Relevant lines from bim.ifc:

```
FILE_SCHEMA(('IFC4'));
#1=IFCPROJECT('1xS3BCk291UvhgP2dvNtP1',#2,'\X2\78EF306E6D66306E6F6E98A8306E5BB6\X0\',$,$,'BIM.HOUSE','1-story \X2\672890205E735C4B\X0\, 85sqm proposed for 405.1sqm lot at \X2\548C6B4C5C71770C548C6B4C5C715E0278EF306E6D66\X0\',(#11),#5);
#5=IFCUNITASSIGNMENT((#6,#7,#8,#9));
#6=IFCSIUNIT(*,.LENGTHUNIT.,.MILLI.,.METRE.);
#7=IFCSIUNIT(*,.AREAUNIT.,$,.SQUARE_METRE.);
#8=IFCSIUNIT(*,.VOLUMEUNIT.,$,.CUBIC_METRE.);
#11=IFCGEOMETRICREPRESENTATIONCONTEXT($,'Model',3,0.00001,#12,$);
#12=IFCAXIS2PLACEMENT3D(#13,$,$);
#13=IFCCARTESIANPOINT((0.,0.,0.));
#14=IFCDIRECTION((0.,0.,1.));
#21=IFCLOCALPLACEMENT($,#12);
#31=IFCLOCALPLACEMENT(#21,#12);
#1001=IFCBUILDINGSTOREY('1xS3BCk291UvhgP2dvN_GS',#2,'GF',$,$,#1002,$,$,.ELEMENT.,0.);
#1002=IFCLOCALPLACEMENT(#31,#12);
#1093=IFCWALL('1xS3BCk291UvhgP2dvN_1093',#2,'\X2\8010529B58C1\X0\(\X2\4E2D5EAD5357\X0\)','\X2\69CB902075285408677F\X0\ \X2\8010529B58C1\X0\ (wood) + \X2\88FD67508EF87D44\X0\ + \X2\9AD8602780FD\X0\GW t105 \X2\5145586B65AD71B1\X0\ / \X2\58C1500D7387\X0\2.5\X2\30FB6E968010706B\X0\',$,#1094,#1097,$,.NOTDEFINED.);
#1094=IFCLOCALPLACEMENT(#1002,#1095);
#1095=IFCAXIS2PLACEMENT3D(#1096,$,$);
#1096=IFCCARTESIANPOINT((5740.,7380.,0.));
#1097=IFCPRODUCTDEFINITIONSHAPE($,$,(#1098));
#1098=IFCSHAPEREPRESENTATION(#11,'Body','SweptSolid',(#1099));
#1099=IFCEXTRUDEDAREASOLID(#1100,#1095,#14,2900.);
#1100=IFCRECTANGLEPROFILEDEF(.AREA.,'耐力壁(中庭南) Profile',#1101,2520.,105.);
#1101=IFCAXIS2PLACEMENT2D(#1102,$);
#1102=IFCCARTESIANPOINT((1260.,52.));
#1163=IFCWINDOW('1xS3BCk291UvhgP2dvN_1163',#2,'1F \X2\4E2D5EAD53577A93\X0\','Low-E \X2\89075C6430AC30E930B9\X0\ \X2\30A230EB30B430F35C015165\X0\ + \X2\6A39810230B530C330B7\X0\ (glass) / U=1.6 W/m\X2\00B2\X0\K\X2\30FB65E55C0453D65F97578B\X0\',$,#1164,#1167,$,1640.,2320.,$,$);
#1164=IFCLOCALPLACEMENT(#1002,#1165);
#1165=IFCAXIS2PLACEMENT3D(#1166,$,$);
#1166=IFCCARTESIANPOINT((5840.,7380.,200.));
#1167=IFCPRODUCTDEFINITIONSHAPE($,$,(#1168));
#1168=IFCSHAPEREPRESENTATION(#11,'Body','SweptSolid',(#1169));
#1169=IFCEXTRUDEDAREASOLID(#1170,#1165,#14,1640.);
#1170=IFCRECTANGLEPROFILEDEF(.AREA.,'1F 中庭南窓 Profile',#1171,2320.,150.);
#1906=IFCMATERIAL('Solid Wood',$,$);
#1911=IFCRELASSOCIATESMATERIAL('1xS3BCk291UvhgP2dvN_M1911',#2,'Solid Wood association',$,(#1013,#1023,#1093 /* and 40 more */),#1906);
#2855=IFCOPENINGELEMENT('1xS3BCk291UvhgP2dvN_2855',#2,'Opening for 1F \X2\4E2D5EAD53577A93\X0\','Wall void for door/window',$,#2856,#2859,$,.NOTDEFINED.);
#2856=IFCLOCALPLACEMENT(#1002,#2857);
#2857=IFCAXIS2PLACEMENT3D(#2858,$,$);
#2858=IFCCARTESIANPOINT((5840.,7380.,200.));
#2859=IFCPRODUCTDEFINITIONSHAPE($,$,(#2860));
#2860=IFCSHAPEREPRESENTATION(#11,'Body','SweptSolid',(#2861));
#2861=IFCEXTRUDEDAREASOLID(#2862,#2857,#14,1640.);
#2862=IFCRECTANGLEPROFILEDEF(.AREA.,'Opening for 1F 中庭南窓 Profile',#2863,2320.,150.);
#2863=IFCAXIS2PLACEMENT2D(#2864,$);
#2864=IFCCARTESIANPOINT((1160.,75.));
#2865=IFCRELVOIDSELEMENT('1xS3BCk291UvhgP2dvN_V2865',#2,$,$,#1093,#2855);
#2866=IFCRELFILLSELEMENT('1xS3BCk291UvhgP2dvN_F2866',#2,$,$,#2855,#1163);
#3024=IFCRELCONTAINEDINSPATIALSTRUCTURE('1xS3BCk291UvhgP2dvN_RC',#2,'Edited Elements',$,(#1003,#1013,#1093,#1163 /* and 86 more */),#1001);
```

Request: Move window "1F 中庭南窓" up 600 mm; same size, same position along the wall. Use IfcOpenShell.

```python
import numpy as np
import ifcopenshell
import ifcopenshell.api.geometry
import ifcopenshell.util.placement
import ifcopenshell.util.unit

model = ifcopenshell.open("bim.ifc")
unit_scale = ifcopenshell.util.unit.calculate_unit_scale(model)

window = model.by_guid("1xS3BCk291UvhgP2dvN_1163")
opening = window.FillsVoids[0].RelatingOpeningElement
dz = 0.6 / unit_scale

shift = np.array([0.0, 0.0, dz])
# The window is not placed relative to its opening, so move both.
for product in (opening, window):
    matrix = ifcopenshell.util.placement.get_local_placement(product.ObjectPlacement)
    matrix[:3, 3] += shift
    ifcopenshell.api.geometry.edit_object_placement(model, product=product, matrix=matrix, is_si=False)

print(f"moved by {dz * unit_scale:+.3f} m")

model.write("bim_edited.ifc")
```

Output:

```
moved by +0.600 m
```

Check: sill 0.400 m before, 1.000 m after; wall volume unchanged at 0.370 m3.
